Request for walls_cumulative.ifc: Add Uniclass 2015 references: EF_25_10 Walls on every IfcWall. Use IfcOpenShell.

First a look at what the model holds.

```python
import ifcopenshell

model = ifcopenshell.open("walls_cumulative.ifc")
print(model.schema)
print("classifications:", [c.Name for c in model.by_type("IfcClassification")])
for ifc_class in ("IfcDoor", "IfcRoof", "IfcStair", "IfcWall", "IfcWindow"):
    print(ifc_class, len(model.by_type(ifc_class)))
```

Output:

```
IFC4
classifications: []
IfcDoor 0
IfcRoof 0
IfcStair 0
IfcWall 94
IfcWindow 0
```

```python
import ifcopenshell
import ifcopenshell.api.classification

model = ifcopenshell.open("walls_cumulative.ifc")

system = ifcopenshell.api.classification.add_classification(model, classification="Uniclass 2015")

codes = {
    "IfcWall": ("EF_25_10", "Walls"),
}
for ifc_class, (code, name) in codes.items():
    products = model.by_type(ifc_class)
    ifcopenshell.api.classification.add_reference(
        model, products=products, classification=system, identification=code, name=name
    )
    print(code, len(products))

model.write("walls_cumulative_edited.ifc")
```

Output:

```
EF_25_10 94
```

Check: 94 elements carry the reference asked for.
